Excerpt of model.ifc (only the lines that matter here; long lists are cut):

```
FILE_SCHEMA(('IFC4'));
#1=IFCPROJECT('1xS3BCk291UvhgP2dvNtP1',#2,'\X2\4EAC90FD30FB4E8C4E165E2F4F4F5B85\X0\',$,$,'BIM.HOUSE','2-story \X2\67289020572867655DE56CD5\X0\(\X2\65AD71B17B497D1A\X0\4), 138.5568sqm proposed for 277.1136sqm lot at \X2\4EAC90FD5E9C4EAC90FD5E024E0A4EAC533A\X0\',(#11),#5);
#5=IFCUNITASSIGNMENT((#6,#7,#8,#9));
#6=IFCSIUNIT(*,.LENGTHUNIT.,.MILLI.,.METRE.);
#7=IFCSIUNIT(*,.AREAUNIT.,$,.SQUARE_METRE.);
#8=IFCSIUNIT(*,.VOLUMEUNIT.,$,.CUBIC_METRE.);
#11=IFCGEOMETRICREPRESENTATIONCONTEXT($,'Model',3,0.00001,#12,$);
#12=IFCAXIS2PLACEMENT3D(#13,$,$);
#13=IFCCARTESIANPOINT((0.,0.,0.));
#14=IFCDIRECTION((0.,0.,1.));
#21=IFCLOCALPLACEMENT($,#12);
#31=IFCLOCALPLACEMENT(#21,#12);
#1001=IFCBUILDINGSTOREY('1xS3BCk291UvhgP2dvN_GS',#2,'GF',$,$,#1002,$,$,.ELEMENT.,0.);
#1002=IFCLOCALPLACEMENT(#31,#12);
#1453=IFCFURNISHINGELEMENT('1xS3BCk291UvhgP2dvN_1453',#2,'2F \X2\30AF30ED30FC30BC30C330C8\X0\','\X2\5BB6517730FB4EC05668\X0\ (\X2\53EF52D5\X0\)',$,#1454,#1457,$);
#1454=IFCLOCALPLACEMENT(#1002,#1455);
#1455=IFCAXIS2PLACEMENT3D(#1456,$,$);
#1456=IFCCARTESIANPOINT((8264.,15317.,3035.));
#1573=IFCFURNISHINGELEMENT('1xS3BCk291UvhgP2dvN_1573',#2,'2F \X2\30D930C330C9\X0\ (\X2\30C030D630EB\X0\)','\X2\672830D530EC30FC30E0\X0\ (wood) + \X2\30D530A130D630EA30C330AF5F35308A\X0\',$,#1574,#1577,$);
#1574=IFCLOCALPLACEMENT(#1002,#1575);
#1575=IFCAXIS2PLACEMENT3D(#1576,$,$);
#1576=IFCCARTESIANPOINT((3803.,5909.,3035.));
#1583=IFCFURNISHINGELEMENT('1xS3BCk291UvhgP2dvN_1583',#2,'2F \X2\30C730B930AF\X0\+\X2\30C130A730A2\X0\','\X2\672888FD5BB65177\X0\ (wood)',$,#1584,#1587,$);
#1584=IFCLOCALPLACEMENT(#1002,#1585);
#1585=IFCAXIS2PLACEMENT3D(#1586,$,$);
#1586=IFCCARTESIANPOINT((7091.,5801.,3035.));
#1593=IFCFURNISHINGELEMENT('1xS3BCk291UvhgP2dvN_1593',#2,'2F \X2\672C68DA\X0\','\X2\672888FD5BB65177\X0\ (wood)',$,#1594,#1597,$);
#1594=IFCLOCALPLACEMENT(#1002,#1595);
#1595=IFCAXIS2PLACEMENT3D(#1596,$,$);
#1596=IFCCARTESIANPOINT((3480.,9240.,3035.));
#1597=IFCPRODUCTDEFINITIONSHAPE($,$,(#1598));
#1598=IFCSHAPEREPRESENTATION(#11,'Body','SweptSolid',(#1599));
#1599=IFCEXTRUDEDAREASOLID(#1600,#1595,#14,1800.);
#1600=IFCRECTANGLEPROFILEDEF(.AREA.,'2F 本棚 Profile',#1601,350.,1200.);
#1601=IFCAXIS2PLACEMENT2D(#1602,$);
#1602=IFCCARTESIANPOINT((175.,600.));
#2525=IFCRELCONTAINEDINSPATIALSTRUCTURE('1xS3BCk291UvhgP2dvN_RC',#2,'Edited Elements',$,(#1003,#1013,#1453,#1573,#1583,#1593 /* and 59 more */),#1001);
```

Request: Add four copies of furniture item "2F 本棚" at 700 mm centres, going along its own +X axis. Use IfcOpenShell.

```python
import ifcopenshell
import ifcopenshell.api.geometry
import ifcopenshell.api.root
import ifcopenshell.util.element
import ifcopenshell.util.placement

model = ifcopenshell.open("model.ifc")


def reuse_history(source, copy):
    """copy_class also copies each property set's owner history, people and application; keep the originals."""
    for rel in copy.IsDefinedBy:
        if rel.is_a("IfcRelDefinesByProperties") and (history := rel.RelatingPropertyDefinition.OwnerHistory):
            rel.RelatingPropertyDefinition.OwnerHistory = source.OwnerHistory
            ifcopenshell.util.element.remove_deep2(model, history)


source = model.by_guid("1xS3BCk291UvhgP2dvN_1593")
base = ifcopenshell.util.placement.get_local_placement(source.ObjectPlacement)
step = base[:3, 0] * 700.0

for i in range(1, 5):
    copy = ifcopenshell.api.root.copy_class(model, product=source)
    copy.Representation = ifcopenshell.util.element.copy_deep(
        model, source.Representation, exclude=["IfcGeometricRepresentationContext", "IfcRepresentationMap"]
    )
    reuse_history(source, copy)
    matrix = base.copy()
    matrix[:3, 3] += i * step
    print("added at", matrix[:3, 3].round(3) + 0.0)
    ifcopenshell.api.geometry.edit_object_placement(model, product=copy, matrix=matrix, is_si=False)

model.write("model_edited.ifc")
```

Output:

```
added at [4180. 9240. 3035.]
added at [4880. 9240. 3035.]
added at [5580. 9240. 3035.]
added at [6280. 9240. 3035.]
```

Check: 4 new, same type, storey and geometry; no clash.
